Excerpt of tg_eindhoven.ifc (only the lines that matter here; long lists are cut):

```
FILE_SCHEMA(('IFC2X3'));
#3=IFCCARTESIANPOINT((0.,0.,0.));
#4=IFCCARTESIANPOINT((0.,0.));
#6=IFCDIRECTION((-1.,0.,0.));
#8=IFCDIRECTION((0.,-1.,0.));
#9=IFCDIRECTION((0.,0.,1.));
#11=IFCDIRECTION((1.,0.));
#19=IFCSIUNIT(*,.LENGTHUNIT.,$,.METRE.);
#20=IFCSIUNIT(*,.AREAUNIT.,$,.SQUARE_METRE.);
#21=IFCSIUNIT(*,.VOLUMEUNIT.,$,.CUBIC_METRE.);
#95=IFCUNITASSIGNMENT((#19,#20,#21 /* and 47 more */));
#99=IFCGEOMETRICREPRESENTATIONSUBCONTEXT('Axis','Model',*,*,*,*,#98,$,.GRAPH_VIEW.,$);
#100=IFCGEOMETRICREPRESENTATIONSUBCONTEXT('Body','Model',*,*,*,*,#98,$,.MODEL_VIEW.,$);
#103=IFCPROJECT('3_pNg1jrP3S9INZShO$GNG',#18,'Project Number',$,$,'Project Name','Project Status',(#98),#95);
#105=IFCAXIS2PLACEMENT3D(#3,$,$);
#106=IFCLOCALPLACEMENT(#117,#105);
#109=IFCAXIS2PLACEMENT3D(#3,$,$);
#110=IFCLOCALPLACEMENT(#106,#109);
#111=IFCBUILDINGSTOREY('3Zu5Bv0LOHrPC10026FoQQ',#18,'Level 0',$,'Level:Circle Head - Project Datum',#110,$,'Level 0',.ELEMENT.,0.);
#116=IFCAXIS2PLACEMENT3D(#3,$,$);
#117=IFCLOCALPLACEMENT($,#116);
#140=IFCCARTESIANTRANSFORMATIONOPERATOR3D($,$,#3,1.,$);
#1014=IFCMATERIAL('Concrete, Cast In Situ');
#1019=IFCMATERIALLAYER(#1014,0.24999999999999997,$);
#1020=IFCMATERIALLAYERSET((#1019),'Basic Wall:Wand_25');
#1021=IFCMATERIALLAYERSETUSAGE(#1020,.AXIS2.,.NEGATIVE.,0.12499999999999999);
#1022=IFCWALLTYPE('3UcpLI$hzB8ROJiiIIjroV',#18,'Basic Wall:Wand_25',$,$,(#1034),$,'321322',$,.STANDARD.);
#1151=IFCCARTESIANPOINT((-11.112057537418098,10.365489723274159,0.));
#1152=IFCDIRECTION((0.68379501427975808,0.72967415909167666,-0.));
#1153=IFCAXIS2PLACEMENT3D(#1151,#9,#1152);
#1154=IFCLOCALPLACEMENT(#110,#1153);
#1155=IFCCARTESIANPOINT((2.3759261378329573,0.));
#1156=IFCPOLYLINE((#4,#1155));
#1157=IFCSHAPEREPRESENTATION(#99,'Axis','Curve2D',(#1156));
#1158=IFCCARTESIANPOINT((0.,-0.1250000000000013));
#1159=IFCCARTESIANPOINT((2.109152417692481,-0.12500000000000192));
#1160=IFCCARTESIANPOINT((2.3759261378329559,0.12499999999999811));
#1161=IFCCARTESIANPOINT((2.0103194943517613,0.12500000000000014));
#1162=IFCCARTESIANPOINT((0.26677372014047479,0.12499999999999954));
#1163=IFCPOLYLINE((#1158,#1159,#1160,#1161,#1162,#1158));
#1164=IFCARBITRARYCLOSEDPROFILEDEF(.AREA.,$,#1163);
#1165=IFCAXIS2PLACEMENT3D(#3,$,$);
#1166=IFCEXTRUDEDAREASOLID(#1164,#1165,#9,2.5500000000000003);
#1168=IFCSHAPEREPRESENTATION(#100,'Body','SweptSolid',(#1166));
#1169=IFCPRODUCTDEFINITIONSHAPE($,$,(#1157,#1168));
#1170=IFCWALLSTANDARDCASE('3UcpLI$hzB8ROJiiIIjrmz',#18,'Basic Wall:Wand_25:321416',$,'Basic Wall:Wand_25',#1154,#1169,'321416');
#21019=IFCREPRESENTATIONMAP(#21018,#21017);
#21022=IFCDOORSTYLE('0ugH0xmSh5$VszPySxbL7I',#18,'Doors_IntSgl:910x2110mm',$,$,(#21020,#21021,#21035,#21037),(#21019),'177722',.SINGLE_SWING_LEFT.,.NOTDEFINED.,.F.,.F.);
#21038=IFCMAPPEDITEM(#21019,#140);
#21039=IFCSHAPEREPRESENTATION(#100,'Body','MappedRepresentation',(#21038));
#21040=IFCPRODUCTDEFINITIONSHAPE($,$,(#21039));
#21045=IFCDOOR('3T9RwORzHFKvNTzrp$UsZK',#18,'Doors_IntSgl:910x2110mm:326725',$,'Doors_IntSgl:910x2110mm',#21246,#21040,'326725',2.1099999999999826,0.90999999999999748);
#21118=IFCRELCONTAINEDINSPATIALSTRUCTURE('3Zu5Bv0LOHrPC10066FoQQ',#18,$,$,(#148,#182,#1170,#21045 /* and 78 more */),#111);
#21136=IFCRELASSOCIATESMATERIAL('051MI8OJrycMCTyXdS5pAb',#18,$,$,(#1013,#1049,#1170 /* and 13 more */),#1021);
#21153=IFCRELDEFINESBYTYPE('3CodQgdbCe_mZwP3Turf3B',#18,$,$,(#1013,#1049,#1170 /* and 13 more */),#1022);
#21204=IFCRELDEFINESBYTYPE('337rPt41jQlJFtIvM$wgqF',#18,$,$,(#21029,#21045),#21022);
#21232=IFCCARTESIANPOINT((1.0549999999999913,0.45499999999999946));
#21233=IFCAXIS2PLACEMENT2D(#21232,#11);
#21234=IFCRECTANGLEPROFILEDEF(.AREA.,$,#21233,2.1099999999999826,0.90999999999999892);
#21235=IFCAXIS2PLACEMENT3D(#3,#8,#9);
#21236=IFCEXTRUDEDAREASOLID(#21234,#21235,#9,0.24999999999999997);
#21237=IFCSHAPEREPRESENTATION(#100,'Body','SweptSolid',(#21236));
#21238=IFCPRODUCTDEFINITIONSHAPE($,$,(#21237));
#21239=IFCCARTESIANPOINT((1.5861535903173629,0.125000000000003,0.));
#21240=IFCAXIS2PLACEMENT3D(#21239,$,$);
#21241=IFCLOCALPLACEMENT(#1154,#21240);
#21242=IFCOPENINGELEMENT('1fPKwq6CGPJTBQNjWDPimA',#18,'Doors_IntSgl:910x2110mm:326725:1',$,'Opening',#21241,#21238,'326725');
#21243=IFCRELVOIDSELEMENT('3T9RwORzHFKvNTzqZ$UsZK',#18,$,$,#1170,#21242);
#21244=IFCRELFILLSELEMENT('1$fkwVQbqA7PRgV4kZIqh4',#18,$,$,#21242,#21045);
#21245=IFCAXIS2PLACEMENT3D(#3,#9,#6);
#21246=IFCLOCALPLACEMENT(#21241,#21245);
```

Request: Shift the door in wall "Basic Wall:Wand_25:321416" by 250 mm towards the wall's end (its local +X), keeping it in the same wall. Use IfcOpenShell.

```python
import ifcopenshell
import ifcopenshell.api.geometry
import ifcopenshell.util.placement
import ifcopenshell.util.unit

model = ifcopenshell.open("tg_eindhoven.ifc")
unit_scale = ifcopenshell.util.unit.calculate_unit_scale(model)

door = model.by_guid("3T9RwORzHFKvNTzrp$UsZK")
opening = door.FillsVoids[0].RelatingOpeningElement
wall = opening.VoidsElements[0].RelatingBuildingElement

wall_matrix = ifcopenshell.util.placement.get_local_placement(wall.ObjectPlacement)
shift = wall_matrix[:3, 0] * 0.25 / unit_scale
before = ifcopenshell.util.placement.get_local_placement(door.ObjectPlacement)[:3, 3].copy()

# The door is placed relative to its opening, so it follows when the opening moves.
matrix = ifcopenshell.util.placement.get_local_placement(opening.ObjectPlacement)
matrix[:3, 3] += shift
ifcopenshell.api.geometry.edit_object_placement(
    model, product=opening, matrix=matrix, is_si=False, should_transform_children=True
)

after = ifcopenshell.util.placement.get_local_placement(door.ObjectPlacement)[:3, 3]
print("door moved by", (after - before).round(3) + 0.0)

model.write("tg_eindhoven_updated.ifc")
```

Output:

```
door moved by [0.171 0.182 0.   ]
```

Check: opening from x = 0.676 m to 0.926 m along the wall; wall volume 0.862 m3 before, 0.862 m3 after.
